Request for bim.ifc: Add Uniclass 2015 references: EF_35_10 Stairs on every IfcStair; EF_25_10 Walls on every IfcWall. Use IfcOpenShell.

First a look at what the model holds.

```python
import ifcopenshell

model = ifcopenshell.open("bim.ifc")
print(model.schema)
print("classifications:", [c.Name for c in model.by_type("IfcClassification")])
for ifc_class in ("IfcDoor", "IfcRoof", "IfcStair", "IfcWall", "IfcWindow"):
    print(ifc_class, len(model.by_type(ifc_class)))
```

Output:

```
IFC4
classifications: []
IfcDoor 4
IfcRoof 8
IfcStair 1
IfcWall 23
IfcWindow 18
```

```python
import ifcopenshell
import ifcopenshell.api.classification

model = ifcopenshell.open("bim.ifc")

system = ifcopenshell.api.classification.add_classification(model, classification="Uniclass 2015")

codes = {
    "IfcStair": ("EF_35_10", "Stairs"),
    "IfcWall": ("EF_25_10", "Walls"),
}
for ifc_class, (code, name) in codes.items():
    products = model.by_type(ifc_class)
    ifcopenshell.api.classification.add_reference(
        model, products=products, classification=system, identification=code, name=name
    )
    print(code, len(products))

model.write("bim_rev.ifc")
```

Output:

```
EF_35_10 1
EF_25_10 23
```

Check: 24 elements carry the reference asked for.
